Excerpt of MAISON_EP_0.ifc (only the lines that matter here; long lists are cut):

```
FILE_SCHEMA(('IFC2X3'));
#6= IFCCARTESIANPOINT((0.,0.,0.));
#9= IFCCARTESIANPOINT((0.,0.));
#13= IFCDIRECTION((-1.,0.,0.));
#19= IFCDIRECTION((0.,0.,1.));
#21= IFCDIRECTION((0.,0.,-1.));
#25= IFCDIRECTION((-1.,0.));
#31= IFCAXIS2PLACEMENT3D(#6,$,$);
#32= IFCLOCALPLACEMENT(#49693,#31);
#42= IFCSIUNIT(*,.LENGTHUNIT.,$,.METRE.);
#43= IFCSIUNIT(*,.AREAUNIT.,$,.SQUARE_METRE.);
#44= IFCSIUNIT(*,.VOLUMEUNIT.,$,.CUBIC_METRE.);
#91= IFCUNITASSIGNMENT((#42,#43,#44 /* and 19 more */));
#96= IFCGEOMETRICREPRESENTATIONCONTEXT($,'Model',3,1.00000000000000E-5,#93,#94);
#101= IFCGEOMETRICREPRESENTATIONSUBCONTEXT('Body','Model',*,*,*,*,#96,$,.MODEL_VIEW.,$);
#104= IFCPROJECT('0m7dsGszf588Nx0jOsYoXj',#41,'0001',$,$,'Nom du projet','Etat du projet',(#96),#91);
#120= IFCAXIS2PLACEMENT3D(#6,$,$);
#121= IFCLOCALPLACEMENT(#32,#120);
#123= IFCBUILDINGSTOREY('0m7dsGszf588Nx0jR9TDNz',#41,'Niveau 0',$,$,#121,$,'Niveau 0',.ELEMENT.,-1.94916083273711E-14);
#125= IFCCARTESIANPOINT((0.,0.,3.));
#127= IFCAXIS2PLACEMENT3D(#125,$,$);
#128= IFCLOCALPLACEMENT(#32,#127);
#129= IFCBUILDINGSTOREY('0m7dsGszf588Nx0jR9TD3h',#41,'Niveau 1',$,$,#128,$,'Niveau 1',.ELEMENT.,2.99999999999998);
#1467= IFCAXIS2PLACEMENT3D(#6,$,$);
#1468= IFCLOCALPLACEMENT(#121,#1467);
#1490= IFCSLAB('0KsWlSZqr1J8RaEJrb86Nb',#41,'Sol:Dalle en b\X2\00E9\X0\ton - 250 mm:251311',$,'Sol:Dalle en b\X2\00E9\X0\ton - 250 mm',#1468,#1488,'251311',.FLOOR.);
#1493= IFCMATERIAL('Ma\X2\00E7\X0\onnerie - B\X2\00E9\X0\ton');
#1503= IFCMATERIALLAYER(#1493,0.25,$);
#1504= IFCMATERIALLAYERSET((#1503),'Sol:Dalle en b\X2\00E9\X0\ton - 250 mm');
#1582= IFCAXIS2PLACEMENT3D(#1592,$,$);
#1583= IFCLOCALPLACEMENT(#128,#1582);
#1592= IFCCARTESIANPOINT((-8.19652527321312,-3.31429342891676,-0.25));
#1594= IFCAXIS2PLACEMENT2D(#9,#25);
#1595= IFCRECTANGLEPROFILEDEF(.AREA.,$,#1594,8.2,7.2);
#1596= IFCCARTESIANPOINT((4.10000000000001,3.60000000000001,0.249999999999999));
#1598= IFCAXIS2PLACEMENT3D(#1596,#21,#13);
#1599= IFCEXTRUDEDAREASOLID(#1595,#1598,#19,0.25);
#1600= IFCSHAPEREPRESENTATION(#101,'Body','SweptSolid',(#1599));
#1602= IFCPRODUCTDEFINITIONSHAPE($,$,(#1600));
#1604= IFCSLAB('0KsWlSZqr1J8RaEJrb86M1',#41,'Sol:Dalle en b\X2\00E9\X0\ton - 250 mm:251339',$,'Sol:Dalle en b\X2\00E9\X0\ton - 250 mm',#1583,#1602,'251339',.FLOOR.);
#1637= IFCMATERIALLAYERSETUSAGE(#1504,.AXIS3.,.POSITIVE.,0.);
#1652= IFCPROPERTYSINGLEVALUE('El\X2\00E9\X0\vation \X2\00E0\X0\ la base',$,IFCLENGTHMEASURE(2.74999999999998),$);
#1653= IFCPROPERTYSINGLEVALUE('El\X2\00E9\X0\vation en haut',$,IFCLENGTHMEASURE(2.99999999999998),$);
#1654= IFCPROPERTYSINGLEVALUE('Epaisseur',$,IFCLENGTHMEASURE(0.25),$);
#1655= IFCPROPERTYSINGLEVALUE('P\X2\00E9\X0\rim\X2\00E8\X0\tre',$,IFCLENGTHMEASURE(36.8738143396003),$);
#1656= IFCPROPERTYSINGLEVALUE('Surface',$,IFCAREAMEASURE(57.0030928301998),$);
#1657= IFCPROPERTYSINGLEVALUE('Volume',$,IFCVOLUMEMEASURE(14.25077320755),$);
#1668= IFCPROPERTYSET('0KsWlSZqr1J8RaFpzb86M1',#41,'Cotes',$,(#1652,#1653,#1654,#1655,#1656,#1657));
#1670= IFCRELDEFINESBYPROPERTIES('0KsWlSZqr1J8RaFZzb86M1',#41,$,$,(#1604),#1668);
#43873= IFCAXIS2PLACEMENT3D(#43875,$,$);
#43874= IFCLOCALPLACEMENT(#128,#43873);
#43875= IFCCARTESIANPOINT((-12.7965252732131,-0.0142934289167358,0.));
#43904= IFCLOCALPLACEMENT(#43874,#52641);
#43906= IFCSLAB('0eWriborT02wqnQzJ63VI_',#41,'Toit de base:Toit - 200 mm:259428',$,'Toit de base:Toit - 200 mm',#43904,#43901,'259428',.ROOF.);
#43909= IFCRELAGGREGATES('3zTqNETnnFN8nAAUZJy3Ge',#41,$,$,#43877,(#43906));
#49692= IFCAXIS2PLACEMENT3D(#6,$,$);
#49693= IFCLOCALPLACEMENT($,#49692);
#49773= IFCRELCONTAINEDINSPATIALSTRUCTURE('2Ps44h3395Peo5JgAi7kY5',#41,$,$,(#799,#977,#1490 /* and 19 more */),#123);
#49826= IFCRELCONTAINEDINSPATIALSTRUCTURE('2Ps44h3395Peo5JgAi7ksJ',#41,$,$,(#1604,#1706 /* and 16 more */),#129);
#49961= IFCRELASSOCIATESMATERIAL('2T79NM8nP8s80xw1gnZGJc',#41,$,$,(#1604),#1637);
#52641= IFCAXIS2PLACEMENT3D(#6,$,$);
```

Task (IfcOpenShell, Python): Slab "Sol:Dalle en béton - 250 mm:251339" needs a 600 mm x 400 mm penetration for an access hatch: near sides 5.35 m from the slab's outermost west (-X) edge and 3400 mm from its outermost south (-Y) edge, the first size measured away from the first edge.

```python
import numpy as np
import ifcopenshell
import ifcopenshell.api.feature
import ifcopenshell.api.geometry
import ifcopenshell.api.pset
import ifcopenshell.api.root
import ifcopenshell.geom
import ifcopenshell.util.element
import ifcopenshell.util.placement
import ifcopenshell.util.representation
import ifcopenshell.util.shape
import ifcopenshell.util.unit

model = ifcopenshell.open("MAISON_EP_0.ifc")
unit_scale = ifcopenshell.util.unit.calculate_unit_scale(model)
area_scale = ifcopenshell.util.unit.calculate_unit_scale(model, "AREAUNIT")
volume_scale = ifcopenshell.util.unit.calculate_unit_scale(model, "VOLUMEUNIT")
settings = ifcopenshell.geom.settings()


def volume(element):
    """Net volume in cubic metres, openings subtracted."""
    shape = ifcopenshell.geom.create_shape(settings, element)
    return ifcopenshell.util.shape.get_volume(shape.geometry)


slab = model.by_id(1604)
before = volume(slab)

# Extent in the slab's own axes, in metres. The edges named are its -X and -Y sides.
slab_shape = ifcopenshell.geom.create_shape(settings, slab)
vertices = ifcopenshell.util.shape.get_vertices(slab_shape.geometry)
x_min, y_min, bottom = vertices.min(axis=0)
top = vertices[:, 2].max()

opening = ifcopenshell.api.root.create_entity(model, ifc_class="IfcOpeningElement", name="Access hatch opening")
context = ifcopenshell.util.representation.get_context(model, "Model", "Body", "MODEL_VIEW")
width, depth = 0.6, 0.4
outline = [(0.0, 0.0), (width, 0.0), (width, depth), (0.0, depth), (0.0, 0.0)]
# Overshoot both faces by 50 mm so the cut is clean.
shape = ifcopenshell.api.geometry.add_slab_representation(
    model, context=context, depth=top - bottom + 0.1, polyline=outline
)
ifcopenshell.api.geometry.assign_representation(model, product=opening, representation=shape)

matrix = ifcopenshell.util.placement.get_local_placement(slab.ObjectPlacement)
matrix[:, 3] = matrix @ np.append(np.array([x_min + 5.35, y_min + 3.4, bottom - 0.05]) / unit_scale, 1.0)
ifcopenshell.api.geometry.edit_object_placement(model, product=opening, matrix=matrix, is_si=False)
ifcopenshell.api.feature.add_feature(model, feature=opening, element=slab)

after = volume(slab)

# Update the slab's stored quantities.
pset = model.by_id(ifcopenshell.util.element.get_pset(slab, "Cotes", should_inherit=False)["id"])
ifcopenshell.api.pset.edit_pset(model, pset=pset, properties={
    "Surface": model.create_entity("IfcAreaMeasure", after / (top - bottom) / area_scale),
    "Volume": model.create_entity("IfcVolumeMeasure", after / volume_scale),
})

print(f"slab volume {before:.3f} -> {after:.3f} m3")

model.write("MAISON_EP_0_updated.ifc")
```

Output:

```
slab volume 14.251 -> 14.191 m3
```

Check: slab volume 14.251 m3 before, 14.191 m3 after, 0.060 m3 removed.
